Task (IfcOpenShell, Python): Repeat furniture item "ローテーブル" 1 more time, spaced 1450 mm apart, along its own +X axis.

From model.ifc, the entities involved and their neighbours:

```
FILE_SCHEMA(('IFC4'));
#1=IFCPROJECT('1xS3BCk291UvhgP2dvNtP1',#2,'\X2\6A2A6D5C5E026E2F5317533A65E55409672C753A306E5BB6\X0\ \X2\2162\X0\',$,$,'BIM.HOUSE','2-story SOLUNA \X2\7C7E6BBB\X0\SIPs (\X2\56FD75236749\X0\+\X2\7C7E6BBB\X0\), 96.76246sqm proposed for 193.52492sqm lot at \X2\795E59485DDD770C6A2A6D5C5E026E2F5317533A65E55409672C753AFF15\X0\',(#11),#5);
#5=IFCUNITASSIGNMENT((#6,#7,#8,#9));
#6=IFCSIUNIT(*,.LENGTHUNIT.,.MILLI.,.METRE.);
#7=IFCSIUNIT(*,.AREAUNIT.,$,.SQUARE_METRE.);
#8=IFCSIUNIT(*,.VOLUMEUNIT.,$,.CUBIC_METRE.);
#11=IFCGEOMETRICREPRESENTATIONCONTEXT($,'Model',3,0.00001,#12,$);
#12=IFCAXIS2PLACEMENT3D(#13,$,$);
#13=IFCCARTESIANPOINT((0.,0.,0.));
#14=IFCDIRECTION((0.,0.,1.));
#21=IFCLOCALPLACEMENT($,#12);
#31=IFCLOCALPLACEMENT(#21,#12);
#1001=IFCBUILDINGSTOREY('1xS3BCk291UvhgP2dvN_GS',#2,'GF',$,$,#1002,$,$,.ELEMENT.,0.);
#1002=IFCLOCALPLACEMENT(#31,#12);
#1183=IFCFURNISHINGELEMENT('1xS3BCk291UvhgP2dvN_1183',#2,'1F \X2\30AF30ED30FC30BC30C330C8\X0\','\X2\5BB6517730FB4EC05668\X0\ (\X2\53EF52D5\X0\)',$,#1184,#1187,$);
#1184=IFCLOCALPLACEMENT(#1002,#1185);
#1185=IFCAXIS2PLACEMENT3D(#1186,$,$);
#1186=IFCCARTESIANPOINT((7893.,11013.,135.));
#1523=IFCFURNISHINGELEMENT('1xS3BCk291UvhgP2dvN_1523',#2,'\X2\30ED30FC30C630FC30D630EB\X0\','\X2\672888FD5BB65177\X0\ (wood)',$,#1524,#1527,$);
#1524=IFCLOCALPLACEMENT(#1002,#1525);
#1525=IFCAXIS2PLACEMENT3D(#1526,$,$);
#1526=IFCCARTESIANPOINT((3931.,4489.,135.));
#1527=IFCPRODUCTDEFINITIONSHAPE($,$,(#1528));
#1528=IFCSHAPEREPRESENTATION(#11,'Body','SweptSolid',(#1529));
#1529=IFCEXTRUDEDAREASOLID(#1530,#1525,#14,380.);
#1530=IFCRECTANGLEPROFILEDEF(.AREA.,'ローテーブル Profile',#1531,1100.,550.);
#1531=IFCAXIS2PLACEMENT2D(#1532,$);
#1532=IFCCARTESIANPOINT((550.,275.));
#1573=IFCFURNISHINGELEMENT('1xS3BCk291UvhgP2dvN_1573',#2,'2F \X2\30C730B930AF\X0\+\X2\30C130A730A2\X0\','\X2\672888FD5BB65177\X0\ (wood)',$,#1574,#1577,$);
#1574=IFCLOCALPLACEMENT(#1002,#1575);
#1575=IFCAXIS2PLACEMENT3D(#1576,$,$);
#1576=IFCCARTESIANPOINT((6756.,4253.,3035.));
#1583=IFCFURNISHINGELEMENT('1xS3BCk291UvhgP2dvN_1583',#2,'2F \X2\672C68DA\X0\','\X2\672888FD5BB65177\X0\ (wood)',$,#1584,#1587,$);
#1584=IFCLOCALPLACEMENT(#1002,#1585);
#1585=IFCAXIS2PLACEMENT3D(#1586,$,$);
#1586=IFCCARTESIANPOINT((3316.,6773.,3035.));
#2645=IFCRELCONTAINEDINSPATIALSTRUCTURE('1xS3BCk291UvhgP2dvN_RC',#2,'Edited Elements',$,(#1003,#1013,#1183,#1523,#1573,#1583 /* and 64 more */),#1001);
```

```python
import ifcopenshell
import ifcopenshell.api.geometry
import ifcopenshell.api.root
import ifcopenshell.util.element
import ifcopenshell.util.placement
import ifcopenshell.util.unit

model = ifcopenshell.open("model.ifc")
unit_scale = ifcopenshell.util.unit.calculate_unit_scale(model)


def reuse_history(source, copy):
    """copy_class also copies each property set's owner history, people and application; keep the originals."""
    for rel in copy.IsDefinedBy:
        if rel.is_a("IfcRelDefinesByProperties") and (history := rel.RelatingPropertyDefinition.OwnerHistory):
            rel.RelatingPropertyDefinition.OwnerHistory = source.OwnerHistory
            ifcopenshell.util.element.remove_deep2(model, history)


source = model.by_guid("1xS3BCk291UvhgP2dvN_1523")
base = ifcopenshell.util.placement.get_local_placement(source.ObjectPlacement)
step = base[:3, 0] * 1.45 / unit_scale

for i in range(1, 2):
    copy = ifcopenshell.api.root.copy_class(model, product=source)
    copy.Representation = ifcopenshell.util.element.copy_deep(
        model, source.Representation, exclude=["IfcGeometricRepresentationContext", "IfcRepresentationMap"]
    )
    reuse_history(source, copy)
    matrix = base.copy()
    matrix[:3, 3] += i * step
    print("added at", matrix[:3, 3].round(3) + 0.0)
    ifcopenshell.api.geometry.edit_object_placement(model, product=copy, matrix=matrix, is_si=False)

model.write("model_rev.ifc")
```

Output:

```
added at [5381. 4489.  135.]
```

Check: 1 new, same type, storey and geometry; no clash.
